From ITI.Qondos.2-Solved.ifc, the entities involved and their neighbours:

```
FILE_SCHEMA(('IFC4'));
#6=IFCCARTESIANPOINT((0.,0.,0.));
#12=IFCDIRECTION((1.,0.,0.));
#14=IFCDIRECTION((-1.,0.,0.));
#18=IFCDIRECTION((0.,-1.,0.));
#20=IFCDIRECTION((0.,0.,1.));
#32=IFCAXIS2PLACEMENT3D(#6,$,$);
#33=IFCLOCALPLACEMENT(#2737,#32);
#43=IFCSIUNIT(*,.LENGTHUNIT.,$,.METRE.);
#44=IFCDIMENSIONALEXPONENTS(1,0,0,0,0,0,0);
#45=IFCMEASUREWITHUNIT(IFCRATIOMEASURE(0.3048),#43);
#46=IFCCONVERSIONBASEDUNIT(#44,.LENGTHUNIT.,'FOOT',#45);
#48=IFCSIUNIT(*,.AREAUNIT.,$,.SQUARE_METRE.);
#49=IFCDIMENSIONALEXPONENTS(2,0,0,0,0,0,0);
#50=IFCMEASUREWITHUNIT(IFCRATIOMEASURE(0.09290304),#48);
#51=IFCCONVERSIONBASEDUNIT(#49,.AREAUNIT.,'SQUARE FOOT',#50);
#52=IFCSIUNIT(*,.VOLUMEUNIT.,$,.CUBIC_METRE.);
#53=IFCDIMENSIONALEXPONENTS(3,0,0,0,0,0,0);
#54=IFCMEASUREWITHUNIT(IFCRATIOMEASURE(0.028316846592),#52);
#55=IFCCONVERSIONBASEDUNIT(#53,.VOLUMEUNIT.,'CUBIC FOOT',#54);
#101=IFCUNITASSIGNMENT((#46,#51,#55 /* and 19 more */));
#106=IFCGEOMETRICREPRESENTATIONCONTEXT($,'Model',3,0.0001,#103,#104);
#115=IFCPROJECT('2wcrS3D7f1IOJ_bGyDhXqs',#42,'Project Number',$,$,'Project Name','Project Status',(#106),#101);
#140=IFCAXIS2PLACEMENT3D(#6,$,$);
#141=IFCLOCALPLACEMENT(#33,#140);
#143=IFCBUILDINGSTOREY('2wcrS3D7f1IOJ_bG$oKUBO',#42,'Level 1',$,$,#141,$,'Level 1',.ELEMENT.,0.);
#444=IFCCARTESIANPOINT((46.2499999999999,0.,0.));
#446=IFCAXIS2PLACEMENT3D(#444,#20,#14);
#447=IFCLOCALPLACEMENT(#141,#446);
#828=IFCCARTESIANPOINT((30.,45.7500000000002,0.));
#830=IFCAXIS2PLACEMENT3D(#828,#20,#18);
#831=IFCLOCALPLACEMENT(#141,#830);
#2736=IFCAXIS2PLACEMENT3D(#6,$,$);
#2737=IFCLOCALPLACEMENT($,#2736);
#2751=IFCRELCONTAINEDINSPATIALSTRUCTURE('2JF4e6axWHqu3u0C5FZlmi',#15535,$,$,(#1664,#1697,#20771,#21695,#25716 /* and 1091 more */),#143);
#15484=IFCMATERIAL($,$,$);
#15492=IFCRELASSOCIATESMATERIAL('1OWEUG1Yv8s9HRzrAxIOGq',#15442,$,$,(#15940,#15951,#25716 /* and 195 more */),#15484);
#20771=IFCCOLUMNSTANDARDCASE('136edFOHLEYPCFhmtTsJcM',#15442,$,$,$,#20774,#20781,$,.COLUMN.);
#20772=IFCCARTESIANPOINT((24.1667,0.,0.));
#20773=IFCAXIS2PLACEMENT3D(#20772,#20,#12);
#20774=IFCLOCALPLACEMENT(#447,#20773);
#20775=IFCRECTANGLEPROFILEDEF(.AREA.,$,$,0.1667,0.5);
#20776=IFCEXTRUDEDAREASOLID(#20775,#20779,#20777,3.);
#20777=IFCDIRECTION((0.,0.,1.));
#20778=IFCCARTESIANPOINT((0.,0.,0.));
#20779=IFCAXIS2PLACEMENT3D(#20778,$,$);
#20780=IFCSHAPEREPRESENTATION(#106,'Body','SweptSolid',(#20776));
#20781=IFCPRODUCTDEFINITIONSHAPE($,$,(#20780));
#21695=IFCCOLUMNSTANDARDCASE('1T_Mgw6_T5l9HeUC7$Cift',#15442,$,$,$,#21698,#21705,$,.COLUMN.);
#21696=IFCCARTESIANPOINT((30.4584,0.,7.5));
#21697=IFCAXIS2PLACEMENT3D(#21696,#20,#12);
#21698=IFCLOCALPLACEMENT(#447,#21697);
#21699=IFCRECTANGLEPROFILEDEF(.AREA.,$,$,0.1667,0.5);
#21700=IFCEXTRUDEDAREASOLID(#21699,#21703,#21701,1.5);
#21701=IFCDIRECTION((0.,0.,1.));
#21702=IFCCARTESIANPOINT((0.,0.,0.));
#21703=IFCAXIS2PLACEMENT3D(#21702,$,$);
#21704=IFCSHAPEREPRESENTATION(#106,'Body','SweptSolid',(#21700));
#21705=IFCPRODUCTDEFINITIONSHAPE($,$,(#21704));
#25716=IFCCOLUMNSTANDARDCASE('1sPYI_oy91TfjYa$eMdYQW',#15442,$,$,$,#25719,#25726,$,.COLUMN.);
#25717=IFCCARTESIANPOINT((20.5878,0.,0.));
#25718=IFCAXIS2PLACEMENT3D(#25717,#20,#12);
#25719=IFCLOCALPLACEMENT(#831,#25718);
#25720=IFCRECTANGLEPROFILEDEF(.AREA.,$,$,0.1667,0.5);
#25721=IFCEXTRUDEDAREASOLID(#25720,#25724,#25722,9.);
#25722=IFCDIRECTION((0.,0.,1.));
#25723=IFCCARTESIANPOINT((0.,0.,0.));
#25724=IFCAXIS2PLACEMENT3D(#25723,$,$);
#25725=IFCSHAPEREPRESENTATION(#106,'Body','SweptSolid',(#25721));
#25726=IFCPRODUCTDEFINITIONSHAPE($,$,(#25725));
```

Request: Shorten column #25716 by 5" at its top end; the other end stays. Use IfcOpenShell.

```python
import ifcopenshell
import ifcopenshell.util.unit

model = ifcopenshell.open("ITI.Qondos.2-Solved.ifc")
unit_scale = ifcopenshell.util.unit.calculate_unit_scale(model)

member = model.by_id(25716)
change = -5 * 0.0254 / unit_scale

# The extrusion runs towards the end named, so only its depth changes.
body = next(r for r in member.Representation.Representations if r.RepresentationIdentifier == "Body")
solid = body.Items[0]
old_length = solid.Depth
solid.Depth += change

print(f"length {old_length:g} -> {solid.Depth:g}")

model.write("ITI.Qondos.2-Solved_rev.ifc")
```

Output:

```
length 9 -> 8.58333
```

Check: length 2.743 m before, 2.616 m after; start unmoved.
